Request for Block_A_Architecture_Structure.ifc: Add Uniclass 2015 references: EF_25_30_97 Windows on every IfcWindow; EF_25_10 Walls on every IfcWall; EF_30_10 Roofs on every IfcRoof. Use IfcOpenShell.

First a look at what the model holds.

```python
import ifcopenshell

model = ifcopenshell.open("Block_A_Architecture_Structure.ifc")
print(model.schema)
print("classifications:", [c.Name for c in model.by_type("IfcClassification")])
for ifc_class in ("IfcDoor", "IfcRoof", "IfcStair", "IfcWall", "IfcWindow"):
    print(ifc_class, len(model.by_type(ifc_class)))
```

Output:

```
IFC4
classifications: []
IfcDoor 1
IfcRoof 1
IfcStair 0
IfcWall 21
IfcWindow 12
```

```python
import ifcopenshell
import ifcopenshell.api.classification

model = ifcopenshell.open("Block_A_Architecture_Structure.ifc")

system = ifcopenshell.api.classification.add_classification(model, classification="Uniclass 2015")

codes = {
    "IfcWindow": ("EF_25_30_97", "Windows"),
    "IfcWall": ("EF_25_10", "Walls"),
    "IfcRoof": ("EF_30_10", "Roofs"),
}
for ifc_class, (code, name) in codes.items():
    products = model.by_type(ifc_class)
    ifcopenshell.api.classification.add_reference(
        model, products=products, classification=system, identification=code, name=name
    )
    print(code, len(products))

model.write("Block_A_Architecture_Structure_v2.ifc")
```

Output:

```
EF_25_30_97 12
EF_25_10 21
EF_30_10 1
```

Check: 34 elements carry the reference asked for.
